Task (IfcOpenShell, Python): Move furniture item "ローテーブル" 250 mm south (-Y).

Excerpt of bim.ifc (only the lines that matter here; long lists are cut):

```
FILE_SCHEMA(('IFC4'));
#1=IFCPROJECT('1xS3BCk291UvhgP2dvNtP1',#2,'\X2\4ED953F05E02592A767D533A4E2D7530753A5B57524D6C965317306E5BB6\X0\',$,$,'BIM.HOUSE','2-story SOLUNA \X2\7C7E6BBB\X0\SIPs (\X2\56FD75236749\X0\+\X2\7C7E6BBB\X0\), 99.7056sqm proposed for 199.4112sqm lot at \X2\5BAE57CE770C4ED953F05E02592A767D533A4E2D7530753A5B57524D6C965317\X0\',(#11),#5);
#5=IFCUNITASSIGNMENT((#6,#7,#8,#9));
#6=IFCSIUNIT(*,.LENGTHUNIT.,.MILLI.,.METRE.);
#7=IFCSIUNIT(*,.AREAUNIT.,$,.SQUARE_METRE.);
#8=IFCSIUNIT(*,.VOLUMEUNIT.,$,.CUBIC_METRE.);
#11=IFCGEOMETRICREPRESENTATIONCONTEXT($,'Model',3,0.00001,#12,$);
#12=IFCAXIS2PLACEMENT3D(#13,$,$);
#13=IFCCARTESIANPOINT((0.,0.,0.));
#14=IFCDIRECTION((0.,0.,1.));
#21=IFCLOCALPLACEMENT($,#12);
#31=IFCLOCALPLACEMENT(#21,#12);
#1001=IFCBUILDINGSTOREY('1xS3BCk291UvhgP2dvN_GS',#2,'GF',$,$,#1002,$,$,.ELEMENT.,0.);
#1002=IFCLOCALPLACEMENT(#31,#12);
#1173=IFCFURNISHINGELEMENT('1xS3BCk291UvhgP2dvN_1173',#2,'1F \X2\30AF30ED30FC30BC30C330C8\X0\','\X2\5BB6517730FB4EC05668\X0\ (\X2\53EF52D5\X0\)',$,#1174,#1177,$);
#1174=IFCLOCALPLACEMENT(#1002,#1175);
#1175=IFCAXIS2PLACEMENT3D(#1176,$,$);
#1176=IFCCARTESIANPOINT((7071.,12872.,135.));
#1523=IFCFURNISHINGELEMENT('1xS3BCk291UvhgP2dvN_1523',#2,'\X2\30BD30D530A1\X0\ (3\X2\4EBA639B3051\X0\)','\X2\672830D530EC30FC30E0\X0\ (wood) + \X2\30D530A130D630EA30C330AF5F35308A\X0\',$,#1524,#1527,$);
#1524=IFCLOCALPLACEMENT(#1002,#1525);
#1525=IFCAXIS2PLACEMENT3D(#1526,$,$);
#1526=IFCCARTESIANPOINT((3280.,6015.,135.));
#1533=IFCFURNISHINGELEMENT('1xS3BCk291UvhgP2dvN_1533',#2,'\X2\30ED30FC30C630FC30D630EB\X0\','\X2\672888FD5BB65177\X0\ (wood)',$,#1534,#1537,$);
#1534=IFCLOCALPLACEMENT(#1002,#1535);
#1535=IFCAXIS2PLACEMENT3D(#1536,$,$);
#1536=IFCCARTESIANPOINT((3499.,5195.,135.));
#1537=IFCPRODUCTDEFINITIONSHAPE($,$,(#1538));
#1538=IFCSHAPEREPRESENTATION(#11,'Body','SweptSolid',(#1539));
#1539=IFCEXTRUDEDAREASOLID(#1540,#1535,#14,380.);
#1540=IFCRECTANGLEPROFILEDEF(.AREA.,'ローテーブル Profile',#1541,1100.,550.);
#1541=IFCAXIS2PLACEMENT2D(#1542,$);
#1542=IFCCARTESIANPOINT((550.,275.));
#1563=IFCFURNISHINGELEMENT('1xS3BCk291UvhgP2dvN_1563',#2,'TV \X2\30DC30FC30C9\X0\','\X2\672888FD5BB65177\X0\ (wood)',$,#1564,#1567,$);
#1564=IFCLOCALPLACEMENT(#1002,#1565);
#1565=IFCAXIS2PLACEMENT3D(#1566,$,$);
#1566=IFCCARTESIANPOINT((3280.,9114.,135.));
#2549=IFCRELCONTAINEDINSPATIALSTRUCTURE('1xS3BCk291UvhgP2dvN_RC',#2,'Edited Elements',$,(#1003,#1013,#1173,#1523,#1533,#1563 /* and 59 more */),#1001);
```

```python
import ifcopenshell
import ifcopenshell.api.geometry
import ifcopenshell.util.placement

model = ifcopenshell.open("bim.ifc")

item = model.by_guid("1xS3BCk291UvhgP2dvN_1533")
matrix = ifcopenshell.util.placement.get_local_placement(item.ObjectPlacement)
matrix[1, 3] -= 250.0
ifcopenshell.api.geometry.edit_object_placement(model, product=item, matrix=matrix, is_si=False)

print(ifcopenshell.util.placement.get_local_placement(item.ObjectPlacement).round(3) + 0.0)

model.write("bim-out.ifc")
```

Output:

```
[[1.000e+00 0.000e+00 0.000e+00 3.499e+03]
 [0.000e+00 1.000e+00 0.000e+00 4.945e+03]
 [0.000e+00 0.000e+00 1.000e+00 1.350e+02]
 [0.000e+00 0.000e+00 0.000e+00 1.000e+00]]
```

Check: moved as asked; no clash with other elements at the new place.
